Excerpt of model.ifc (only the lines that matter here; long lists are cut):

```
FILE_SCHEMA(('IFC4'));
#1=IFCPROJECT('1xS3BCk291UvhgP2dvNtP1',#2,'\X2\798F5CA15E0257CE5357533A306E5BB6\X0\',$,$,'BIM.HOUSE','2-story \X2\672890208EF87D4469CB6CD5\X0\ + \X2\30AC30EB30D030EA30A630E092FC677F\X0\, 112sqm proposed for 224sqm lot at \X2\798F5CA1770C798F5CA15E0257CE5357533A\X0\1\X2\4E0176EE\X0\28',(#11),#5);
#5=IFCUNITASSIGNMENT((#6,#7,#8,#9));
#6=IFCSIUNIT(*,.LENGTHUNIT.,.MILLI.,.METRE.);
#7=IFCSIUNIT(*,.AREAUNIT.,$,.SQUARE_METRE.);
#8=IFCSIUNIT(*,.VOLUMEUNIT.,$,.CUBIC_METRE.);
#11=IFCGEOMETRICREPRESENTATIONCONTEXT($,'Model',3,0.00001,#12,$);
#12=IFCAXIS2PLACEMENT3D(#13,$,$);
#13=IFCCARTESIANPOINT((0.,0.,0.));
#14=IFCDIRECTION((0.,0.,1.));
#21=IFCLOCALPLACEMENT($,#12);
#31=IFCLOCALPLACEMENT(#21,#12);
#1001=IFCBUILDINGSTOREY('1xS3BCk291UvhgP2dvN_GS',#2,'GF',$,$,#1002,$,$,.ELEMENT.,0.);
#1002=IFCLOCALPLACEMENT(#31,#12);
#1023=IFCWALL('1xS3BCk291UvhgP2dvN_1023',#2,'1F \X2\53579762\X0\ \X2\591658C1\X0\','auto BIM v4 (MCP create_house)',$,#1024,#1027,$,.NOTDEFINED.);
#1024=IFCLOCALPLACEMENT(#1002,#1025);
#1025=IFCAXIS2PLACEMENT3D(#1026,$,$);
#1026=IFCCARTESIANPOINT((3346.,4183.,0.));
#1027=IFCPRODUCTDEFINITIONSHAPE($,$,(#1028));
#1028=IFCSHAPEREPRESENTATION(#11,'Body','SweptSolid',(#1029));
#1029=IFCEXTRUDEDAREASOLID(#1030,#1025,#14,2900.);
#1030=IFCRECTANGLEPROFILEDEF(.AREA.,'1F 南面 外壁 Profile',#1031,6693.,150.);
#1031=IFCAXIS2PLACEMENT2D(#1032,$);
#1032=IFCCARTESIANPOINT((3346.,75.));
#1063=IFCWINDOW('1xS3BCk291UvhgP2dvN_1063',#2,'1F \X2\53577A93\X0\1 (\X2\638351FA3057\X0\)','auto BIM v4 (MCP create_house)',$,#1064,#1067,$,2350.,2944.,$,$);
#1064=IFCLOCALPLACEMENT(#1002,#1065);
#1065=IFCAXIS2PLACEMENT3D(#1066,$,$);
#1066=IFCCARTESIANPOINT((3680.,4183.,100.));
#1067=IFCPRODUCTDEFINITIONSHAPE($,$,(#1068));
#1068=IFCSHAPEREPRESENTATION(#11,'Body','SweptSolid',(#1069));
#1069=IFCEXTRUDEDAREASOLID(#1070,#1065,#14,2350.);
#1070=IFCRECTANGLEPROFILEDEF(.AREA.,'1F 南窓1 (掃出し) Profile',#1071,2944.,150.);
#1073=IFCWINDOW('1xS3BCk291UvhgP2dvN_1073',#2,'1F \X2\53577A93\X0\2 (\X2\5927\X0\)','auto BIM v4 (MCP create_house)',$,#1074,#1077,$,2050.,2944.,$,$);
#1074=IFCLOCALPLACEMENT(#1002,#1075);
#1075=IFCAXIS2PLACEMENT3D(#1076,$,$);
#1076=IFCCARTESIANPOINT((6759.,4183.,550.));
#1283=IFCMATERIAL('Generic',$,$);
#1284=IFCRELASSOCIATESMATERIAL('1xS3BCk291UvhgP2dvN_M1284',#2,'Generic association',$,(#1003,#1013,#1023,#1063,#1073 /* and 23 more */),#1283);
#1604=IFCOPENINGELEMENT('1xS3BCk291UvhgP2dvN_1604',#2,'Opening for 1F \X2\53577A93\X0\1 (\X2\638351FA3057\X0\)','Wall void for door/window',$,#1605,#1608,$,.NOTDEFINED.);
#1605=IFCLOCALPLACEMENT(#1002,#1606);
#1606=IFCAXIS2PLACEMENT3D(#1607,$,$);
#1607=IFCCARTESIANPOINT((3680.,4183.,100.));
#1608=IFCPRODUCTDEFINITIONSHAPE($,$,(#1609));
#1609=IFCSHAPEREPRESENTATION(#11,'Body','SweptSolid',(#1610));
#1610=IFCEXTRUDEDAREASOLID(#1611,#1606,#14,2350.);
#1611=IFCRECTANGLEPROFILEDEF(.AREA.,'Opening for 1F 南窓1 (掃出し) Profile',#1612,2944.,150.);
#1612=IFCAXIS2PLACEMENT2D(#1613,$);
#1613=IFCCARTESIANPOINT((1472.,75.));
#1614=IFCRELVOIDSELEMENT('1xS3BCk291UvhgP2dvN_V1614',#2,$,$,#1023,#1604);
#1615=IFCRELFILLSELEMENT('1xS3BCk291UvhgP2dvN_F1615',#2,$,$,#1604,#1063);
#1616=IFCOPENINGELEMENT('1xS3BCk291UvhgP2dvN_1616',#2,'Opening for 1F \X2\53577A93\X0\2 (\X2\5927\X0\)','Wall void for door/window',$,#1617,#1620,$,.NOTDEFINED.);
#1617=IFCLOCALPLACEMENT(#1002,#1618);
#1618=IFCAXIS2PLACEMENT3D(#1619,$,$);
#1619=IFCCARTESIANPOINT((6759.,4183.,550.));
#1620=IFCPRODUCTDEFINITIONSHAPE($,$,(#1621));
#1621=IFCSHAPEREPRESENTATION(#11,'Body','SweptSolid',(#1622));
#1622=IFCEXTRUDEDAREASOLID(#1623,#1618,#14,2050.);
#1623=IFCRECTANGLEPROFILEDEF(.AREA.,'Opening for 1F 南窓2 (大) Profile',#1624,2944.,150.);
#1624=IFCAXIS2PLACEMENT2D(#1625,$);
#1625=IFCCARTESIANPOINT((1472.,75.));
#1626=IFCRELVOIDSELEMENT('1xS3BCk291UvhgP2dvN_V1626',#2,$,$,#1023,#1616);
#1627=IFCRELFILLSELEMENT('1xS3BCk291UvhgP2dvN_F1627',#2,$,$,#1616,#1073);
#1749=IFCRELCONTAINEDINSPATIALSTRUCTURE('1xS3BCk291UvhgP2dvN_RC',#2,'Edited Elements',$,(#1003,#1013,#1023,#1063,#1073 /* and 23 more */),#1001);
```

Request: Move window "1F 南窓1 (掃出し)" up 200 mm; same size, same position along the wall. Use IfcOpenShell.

```python
import numpy as np
import ifcopenshell
import ifcopenshell.api.geometry
import ifcopenshell.util.placement
import ifcopenshell.util.unit

model = ifcopenshell.open("model.ifc")
unit_scale = ifcopenshell.util.unit.calculate_unit_scale(model)

window = model.by_guid("1xS3BCk291UvhgP2dvN_1063")
opening = window.FillsVoids[0].RelatingOpeningElement
dz = 0.2 / unit_scale

shift = np.array([0.0, 0.0, dz])
# The window is not placed relative to its opening, so move both.
for product in (opening, window):
    matrix = ifcopenshell.util.placement.get_local_placement(product.ObjectPlacement)
    matrix[:3, 3] += shift
    ifcopenshell.api.geometry.edit_object_placement(model, product=product, matrix=matrix, is_si=False)

print(f"moved by {dz * unit_scale:+.3f} m")

model.write("model-out.ifc")
```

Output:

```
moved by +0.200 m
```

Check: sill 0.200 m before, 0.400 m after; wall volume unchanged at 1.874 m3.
